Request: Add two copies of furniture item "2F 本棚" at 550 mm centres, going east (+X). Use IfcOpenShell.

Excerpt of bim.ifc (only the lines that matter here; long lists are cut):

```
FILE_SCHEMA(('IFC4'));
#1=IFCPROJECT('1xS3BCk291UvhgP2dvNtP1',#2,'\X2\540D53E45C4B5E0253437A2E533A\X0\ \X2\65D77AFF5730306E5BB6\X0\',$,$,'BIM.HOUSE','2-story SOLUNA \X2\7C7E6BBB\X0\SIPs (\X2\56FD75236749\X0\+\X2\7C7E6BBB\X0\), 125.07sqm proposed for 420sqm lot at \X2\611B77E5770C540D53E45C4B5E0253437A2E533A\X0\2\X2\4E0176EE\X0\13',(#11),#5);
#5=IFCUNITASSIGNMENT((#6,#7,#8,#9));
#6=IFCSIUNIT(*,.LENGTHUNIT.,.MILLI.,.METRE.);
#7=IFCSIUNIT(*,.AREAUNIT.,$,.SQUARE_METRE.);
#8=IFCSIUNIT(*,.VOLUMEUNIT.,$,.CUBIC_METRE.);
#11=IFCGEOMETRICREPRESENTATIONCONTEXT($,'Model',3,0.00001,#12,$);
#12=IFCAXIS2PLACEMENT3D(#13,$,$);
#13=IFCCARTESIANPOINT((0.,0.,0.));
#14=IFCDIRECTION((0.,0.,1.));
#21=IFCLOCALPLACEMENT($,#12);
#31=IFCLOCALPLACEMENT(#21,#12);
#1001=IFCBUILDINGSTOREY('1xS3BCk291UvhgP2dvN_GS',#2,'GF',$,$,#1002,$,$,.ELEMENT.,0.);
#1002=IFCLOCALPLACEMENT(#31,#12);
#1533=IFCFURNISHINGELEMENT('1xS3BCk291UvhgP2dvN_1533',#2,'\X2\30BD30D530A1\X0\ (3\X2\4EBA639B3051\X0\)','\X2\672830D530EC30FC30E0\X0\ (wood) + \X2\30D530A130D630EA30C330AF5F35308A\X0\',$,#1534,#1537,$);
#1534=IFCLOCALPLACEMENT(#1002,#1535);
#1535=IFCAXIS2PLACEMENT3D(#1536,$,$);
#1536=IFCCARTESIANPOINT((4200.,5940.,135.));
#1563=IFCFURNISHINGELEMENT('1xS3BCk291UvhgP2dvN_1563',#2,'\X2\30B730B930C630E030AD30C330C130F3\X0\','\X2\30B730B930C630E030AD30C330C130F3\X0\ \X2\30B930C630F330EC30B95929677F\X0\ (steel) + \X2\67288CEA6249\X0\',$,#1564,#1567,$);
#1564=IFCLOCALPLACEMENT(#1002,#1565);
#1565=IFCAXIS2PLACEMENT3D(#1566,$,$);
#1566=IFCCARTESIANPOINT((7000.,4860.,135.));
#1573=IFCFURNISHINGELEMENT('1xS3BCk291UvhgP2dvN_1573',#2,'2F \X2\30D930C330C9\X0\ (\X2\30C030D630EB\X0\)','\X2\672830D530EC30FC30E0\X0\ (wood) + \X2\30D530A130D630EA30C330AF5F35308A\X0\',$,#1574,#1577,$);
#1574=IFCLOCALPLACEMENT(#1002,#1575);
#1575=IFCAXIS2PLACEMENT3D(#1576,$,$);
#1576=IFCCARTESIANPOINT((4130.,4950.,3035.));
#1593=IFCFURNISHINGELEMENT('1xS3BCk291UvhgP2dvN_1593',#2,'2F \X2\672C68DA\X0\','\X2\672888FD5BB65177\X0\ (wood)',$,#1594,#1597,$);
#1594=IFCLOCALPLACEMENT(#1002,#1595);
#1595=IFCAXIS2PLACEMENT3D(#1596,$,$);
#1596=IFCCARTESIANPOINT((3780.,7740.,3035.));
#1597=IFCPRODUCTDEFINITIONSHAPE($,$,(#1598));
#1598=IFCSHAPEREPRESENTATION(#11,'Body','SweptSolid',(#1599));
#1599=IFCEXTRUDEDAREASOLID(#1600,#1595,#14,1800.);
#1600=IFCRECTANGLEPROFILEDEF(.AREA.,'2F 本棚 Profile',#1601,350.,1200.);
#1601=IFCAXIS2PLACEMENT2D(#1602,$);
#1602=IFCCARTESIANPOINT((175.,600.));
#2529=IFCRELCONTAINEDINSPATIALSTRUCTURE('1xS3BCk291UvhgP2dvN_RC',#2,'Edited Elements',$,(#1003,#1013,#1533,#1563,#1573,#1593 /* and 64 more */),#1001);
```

```python
import numpy as np
import ifcopenshell
import ifcopenshell.api.geometry
import ifcopenshell.api.root
import ifcopenshell.util.element
import ifcopenshell.util.placement
import ifcopenshell.util.unit

model = ifcopenshell.open("bim.ifc")
unit_scale = ifcopenshell.util.unit.calculate_unit_scale(model)


def reuse_history(source, copy):
    """copy_class also copies each property set's owner history, people and application; keep the originals."""
    for rel in copy.IsDefinedBy:
        if rel.is_a("IfcRelDefinesByProperties") and (history := rel.RelatingPropertyDefinition.OwnerHistory):
            rel.RelatingPropertyDefinition.OwnerHistory = source.OwnerHistory
            ifcopenshell.util.element.remove_deep2(model, history)


source = model.by_guid("1xS3BCk291UvhgP2dvN_1593")
base = ifcopenshell.util.placement.get_local_placement(source.ObjectPlacement)
step = np.array([1.0, 0.0, 0.0]) * 0.55 / unit_scale

for i in range(1, 3):
    copy = ifcopenshell.api.root.copy_class(model, product=source)
    copy.Representation = ifcopenshell.util.element.copy_deep(
        model, source.Representation, exclude=["IfcGeometricRepresentationContext", "IfcRepresentationMap"]
    )
    reuse_history(source, copy)
    matrix = base.copy()
    matrix[:3, 3] += i * step
    print("added at", matrix[:3, 3].round(3) + 0.0)
    ifcopenshell.api.geometry.edit_object_placement(model, product=copy, matrix=matrix, is_si=False)

model.write("bim_rev.ifc")
```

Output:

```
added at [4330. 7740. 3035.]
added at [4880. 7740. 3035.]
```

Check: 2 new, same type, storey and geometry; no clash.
